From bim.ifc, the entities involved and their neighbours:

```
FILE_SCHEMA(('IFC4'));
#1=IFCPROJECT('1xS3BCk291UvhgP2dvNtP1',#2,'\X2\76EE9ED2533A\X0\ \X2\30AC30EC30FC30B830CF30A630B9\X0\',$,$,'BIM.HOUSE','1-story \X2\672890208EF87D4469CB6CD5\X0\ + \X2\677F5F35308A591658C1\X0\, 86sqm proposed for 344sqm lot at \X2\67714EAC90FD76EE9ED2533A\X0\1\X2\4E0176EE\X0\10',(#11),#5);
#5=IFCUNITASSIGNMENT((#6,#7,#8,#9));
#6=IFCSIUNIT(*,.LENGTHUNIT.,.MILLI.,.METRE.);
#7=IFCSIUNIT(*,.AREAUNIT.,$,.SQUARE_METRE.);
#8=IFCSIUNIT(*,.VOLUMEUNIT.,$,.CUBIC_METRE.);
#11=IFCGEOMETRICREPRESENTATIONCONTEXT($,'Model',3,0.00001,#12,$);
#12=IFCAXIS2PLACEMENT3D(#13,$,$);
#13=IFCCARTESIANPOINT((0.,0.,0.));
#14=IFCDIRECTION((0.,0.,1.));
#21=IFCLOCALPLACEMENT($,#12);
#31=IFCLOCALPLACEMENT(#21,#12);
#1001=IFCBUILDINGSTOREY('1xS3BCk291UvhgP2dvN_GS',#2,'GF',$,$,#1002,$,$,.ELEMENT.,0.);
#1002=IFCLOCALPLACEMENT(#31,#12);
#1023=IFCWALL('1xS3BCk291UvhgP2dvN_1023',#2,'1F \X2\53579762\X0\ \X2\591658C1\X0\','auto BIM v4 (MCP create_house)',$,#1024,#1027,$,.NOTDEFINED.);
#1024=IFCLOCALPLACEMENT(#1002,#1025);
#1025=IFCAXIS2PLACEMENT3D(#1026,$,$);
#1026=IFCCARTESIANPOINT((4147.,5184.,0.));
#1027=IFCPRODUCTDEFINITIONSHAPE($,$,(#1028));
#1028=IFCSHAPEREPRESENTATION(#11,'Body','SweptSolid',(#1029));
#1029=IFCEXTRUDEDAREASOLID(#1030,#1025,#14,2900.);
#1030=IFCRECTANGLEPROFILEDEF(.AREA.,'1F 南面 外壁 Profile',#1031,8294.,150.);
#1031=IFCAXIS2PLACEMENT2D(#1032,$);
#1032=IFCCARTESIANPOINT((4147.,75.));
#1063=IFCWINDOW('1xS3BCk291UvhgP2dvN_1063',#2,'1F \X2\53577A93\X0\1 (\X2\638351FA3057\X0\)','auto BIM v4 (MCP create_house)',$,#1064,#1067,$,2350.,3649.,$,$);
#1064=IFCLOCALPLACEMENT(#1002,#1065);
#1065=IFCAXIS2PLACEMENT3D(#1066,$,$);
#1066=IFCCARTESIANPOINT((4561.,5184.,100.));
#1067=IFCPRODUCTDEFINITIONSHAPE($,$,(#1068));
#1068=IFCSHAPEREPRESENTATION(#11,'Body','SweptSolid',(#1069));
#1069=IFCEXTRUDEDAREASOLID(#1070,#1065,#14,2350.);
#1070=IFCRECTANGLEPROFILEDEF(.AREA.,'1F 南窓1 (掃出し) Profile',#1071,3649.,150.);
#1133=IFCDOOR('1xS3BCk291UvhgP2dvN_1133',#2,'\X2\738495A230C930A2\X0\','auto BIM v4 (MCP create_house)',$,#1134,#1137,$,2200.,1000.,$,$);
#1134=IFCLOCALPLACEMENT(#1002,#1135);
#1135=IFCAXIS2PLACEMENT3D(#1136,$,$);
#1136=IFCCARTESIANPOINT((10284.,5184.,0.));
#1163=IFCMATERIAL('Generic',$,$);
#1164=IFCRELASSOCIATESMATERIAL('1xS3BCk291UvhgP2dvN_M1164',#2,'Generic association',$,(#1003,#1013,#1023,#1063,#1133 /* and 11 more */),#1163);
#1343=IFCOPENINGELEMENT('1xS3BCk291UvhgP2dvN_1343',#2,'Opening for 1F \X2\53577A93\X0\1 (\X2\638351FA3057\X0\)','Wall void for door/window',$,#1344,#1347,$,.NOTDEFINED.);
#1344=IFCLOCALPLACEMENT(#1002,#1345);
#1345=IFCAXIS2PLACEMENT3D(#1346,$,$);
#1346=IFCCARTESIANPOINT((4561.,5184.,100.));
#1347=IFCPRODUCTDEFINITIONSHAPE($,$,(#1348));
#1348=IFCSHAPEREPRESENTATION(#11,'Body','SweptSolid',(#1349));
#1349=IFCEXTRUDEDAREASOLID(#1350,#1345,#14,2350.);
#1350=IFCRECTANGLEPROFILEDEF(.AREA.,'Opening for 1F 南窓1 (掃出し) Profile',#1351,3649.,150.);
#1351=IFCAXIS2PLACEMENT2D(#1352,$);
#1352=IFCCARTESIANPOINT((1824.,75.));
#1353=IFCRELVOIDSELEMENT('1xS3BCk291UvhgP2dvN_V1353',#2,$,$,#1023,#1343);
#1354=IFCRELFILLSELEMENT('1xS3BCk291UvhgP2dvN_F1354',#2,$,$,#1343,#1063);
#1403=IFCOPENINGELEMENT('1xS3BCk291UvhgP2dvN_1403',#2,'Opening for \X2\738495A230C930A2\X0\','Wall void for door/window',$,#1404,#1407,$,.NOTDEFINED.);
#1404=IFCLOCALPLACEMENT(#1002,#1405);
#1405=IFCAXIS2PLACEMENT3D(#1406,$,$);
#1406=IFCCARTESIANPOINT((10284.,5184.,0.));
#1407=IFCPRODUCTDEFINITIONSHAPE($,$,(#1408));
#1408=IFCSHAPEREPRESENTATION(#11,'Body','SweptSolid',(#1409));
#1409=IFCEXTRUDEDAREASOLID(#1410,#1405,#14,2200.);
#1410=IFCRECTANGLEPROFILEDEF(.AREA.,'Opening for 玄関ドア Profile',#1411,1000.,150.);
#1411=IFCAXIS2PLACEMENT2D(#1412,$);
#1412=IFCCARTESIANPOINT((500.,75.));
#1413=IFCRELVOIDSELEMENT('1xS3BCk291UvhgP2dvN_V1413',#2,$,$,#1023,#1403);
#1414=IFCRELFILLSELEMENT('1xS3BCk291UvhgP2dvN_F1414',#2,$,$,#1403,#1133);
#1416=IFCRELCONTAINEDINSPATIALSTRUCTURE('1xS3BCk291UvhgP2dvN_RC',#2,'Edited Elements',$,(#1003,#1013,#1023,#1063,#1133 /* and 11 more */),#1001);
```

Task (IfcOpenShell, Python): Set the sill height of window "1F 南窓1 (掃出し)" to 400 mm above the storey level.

```python
import numpy as np
import ifcopenshell
import ifcopenshell.api.geometry
import ifcopenshell.geom
import ifcopenshell.util.element
import ifcopenshell.util.placement
import ifcopenshell.util.shape
import ifcopenshell.util.unit

model = ifcopenshell.open("bim.ifc")
unit_scale = ifcopenshell.util.unit.calculate_unit_scale(model)

window = model.by_guid("1xS3BCk291UvhgP2dvN_1063")
opening = window.FillsVoids[0].RelatingOpeningElement
storey = ifcopenshell.util.element.get_container(window, ifc_class="IfcBuildingStorey")
level = ifcopenshell.util.placement.get_local_placement(storey.ObjectPlacement)[2, 3]

# The opening's origin need not be at the sill, so measure its lowest point.
shape = ifcopenshell.geom.create_shape(ifcopenshell.geom.settings(), opening)
bottom = ifcopenshell.util.shape.get_shape_bottom_elevation(shape, shape.geometry) / unit_scale
dz = level + 400.0 - bottom

shift = np.array([0.0, 0.0, dz])
# The window is not placed relative to its opening, so move both.
for product in (opening, window):
    matrix = ifcopenshell.util.placement.get_local_placement(product.ObjectPlacement)
    matrix[:3, 3] += shift
    ifcopenshell.api.geometry.edit_object_placement(model, product=product, matrix=matrix, is_si=False)

print(f"moved by {dz * unit_scale:+.3f} m")

model.write("bim_rev.ifc")
```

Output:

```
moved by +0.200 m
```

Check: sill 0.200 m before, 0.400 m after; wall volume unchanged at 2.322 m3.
